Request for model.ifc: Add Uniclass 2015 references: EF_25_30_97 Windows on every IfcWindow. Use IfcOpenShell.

First a look at what the model holds.

```python
import ifcopenshell

model = ifcopenshell.open("model.ifc")
print(model.schema)
print("classifications:", [c.Name for c in model.by_type("IfcClassification")])
for ifc_class in ("IfcDoor", "IfcRoof", "IfcStair", "IfcWall", "IfcWindow"):
    print(ifc_class, len(model.by_type(ifc_class)))
```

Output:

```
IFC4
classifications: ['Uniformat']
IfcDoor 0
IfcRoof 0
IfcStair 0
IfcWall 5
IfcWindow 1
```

```python
import ifcopenshell
import ifcopenshell.api.classification

model = ifcopenshell.open("model.ifc")

system = ifcopenshell.api.classification.add_classification(model, classification="Uniclass 2015")

codes = {
    "IfcWindow": ("EF_25_30_97", "Windows"),
}
for ifc_class, (code, name) in codes.items():
    products = model.by_type(ifc_class)
    ifcopenshell.api.classification.add_reference(
        model, products=products, classification=system, identification=code, name=name
    )
    print(code, len(products))

model.write("model_v2.ifc")
```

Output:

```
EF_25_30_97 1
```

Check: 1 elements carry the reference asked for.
